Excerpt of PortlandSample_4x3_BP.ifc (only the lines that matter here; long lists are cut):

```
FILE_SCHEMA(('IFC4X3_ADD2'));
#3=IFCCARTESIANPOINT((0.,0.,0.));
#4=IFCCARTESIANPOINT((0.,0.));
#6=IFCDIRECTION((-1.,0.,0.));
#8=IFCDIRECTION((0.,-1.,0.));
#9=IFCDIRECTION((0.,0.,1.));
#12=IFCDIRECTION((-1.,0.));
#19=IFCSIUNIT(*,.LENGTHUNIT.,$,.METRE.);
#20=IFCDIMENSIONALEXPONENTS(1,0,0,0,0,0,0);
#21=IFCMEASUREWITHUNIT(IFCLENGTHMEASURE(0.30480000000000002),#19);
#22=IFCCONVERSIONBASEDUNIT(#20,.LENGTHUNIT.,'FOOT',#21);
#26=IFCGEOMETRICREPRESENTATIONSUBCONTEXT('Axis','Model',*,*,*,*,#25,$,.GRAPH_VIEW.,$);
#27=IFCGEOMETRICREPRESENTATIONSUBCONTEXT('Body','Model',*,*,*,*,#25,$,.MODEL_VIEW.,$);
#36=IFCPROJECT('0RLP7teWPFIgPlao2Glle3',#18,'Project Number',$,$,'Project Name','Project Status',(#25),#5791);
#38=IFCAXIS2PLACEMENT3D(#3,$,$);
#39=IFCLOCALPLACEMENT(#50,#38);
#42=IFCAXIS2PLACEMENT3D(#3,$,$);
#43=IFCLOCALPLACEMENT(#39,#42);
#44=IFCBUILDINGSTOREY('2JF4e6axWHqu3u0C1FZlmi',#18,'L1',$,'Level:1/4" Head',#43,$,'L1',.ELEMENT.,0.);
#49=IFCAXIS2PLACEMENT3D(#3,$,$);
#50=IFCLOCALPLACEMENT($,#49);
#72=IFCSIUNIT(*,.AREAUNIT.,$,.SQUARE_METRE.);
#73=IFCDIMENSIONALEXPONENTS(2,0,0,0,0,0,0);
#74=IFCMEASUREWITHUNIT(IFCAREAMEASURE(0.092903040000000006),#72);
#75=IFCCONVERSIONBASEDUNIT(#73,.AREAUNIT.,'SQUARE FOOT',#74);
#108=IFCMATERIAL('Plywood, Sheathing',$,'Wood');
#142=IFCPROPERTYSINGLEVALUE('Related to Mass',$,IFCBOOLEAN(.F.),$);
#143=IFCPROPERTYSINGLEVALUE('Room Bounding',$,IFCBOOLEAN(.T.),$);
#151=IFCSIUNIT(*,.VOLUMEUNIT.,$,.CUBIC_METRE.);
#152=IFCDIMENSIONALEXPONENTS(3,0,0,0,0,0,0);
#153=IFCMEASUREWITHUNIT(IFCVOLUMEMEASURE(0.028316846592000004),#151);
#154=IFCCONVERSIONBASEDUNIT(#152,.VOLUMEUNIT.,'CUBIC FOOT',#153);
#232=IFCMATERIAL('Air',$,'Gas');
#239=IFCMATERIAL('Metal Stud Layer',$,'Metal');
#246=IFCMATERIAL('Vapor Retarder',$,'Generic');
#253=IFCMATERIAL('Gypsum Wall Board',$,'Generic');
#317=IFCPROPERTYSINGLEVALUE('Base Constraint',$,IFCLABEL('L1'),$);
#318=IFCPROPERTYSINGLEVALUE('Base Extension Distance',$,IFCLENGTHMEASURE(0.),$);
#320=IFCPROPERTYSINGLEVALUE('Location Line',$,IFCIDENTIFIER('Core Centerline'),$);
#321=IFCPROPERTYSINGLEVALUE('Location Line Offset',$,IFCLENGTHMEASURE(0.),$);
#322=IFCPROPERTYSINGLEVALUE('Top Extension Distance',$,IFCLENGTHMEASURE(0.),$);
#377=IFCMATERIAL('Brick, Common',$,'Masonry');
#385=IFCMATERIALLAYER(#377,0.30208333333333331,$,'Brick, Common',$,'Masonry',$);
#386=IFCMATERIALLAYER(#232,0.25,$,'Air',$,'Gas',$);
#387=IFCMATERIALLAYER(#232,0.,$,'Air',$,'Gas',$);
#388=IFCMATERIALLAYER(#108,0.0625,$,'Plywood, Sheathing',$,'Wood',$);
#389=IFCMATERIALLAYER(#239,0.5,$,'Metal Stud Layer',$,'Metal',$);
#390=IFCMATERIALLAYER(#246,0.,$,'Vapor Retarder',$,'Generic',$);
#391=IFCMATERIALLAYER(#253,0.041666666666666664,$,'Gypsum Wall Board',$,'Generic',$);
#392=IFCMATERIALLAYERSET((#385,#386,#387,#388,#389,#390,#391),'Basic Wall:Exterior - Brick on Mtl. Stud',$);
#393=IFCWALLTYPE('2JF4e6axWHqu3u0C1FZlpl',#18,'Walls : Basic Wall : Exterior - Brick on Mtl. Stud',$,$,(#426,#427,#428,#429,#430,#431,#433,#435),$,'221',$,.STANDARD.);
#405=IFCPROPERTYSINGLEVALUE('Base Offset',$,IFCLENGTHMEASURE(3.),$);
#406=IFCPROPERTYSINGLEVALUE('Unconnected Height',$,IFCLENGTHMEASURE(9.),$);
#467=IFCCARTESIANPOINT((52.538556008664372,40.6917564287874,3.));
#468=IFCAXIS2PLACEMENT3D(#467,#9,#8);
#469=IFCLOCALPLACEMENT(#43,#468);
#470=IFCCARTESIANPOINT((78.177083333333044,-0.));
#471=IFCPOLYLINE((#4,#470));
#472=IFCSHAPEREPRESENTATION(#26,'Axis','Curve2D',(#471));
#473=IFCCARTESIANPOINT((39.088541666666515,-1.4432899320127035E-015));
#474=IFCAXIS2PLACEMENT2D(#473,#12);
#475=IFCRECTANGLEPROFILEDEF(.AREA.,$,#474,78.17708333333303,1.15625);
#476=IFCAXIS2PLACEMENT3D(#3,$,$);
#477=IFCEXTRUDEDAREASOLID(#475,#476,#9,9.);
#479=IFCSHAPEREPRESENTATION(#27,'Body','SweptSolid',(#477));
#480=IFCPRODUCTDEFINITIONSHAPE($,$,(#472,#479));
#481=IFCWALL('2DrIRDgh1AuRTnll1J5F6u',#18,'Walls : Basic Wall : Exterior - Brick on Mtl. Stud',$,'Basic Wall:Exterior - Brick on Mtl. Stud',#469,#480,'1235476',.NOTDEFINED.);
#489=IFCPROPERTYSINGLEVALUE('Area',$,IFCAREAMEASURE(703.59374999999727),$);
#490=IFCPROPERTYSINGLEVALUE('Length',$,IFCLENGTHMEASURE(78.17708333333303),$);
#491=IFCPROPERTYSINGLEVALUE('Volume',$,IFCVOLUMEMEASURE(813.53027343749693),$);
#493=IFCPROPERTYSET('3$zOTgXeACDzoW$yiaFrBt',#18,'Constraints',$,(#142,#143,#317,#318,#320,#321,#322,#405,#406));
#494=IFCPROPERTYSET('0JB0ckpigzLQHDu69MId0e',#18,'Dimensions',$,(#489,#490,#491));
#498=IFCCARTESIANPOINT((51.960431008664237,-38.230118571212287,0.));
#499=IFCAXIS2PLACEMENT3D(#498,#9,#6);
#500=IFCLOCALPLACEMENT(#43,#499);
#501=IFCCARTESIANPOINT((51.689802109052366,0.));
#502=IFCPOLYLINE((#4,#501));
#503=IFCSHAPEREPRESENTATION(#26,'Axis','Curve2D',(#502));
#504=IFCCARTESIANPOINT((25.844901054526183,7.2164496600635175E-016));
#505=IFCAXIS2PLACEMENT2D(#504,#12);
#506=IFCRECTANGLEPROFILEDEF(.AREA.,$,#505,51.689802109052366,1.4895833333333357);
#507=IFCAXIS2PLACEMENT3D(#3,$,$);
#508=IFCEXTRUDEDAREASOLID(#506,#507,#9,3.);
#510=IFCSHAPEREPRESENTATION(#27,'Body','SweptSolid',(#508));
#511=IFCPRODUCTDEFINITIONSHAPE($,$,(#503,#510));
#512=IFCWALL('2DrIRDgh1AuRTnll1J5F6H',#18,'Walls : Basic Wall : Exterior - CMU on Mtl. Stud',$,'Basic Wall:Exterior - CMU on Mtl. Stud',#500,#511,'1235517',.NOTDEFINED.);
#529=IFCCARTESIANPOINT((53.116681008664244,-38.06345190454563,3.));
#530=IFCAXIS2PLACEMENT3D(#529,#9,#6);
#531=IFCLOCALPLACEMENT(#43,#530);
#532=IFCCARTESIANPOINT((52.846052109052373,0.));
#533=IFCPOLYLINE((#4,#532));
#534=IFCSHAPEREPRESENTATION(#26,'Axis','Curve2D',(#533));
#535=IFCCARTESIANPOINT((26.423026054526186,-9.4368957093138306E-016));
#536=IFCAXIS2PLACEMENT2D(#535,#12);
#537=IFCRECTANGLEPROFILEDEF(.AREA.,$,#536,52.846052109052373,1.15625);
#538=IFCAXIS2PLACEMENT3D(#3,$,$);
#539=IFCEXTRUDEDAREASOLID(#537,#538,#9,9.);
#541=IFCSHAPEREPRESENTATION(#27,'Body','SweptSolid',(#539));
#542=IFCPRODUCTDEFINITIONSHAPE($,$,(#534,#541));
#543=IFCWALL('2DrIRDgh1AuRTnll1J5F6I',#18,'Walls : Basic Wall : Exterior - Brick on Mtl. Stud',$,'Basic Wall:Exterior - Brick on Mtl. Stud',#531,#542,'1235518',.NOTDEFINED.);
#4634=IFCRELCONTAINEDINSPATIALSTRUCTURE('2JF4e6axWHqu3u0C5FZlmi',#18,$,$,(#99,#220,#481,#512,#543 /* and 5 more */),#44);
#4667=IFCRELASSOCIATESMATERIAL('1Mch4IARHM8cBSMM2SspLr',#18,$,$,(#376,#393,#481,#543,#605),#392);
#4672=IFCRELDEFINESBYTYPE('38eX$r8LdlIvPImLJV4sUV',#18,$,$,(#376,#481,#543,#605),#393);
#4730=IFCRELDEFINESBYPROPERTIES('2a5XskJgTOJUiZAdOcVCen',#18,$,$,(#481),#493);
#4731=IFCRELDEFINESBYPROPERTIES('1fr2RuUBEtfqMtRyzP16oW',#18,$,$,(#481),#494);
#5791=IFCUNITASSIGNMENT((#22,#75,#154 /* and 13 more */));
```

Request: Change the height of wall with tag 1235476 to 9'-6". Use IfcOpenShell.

```python
import ifcopenshell
import ifcopenshell.api.pset
import ifcopenshell.geom
import ifcopenshell.util.element
import ifcopenshell.util.representation
import ifcopenshell.util.shape
import ifcopenshell.util.unit

model = ifcopenshell.open("PortlandSample_4x3_BP.ifc")
unit_scale = ifcopenshell.util.unit.calculate_unit_scale(model)
area_scale = ifcopenshell.util.unit.calculate_unit_scale(model, "AREAUNIT")
volume_scale = ifcopenshell.util.unit.calculate_unit_scale(model, "VOLUMEUNIT")
settings = ifcopenshell.geom.settings()


def volume(element):
    """Net volume in cubic metres, openings subtracted."""
    shape = ifcopenshell.geom.create_shape(settings, element)
    return ifcopenshell.util.shape.get_volume(shape.geometry)


wall = model.by_guid("2DrIRDgh1AuRTnll1J5F6u")
before = volume(wall)

body = ifcopenshell.util.representation.get_representation(wall, "Model", "Body")
solid = body.Items[0]
old_height = solid.Depth
solid.Depth = 114 * 0.0254 / unit_scale
after = volume(wall)
thickness = 0.3524  # wall thickness in metres

# Update the stored height, areas and volumes.
pset = model.by_id(ifcopenshell.util.element.get_pset(wall, "Constraints", should_inherit=False)["id"])
ifcopenshell.api.pset.edit_pset(model, pset=pset, properties={
    "Unconnected Height": model.create_entity("IfcLengthMeasure", solid.Depth),
})
pset = model.by_id(ifcopenshell.util.element.get_pset(wall, "Dimensions", should_inherit=False)["id"])
ifcopenshell.api.pset.edit_pset(model, pset=pset, properties={
    "Area": model.create_entity("IfcAreaMeasure", after / thickness / area_scale),
    "Volume": model.create_entity("IfcVolumeMeasure", after / volume_scale),
})

print(f"height {old_height:g} -> {solid.Depth:g}, volume {before:.3f} -> {after:.3f} m3")

model.write("PortlandSample_4x3_BP_edited.ifc")
```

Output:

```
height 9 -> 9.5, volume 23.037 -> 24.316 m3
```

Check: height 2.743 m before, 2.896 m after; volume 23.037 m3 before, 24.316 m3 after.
